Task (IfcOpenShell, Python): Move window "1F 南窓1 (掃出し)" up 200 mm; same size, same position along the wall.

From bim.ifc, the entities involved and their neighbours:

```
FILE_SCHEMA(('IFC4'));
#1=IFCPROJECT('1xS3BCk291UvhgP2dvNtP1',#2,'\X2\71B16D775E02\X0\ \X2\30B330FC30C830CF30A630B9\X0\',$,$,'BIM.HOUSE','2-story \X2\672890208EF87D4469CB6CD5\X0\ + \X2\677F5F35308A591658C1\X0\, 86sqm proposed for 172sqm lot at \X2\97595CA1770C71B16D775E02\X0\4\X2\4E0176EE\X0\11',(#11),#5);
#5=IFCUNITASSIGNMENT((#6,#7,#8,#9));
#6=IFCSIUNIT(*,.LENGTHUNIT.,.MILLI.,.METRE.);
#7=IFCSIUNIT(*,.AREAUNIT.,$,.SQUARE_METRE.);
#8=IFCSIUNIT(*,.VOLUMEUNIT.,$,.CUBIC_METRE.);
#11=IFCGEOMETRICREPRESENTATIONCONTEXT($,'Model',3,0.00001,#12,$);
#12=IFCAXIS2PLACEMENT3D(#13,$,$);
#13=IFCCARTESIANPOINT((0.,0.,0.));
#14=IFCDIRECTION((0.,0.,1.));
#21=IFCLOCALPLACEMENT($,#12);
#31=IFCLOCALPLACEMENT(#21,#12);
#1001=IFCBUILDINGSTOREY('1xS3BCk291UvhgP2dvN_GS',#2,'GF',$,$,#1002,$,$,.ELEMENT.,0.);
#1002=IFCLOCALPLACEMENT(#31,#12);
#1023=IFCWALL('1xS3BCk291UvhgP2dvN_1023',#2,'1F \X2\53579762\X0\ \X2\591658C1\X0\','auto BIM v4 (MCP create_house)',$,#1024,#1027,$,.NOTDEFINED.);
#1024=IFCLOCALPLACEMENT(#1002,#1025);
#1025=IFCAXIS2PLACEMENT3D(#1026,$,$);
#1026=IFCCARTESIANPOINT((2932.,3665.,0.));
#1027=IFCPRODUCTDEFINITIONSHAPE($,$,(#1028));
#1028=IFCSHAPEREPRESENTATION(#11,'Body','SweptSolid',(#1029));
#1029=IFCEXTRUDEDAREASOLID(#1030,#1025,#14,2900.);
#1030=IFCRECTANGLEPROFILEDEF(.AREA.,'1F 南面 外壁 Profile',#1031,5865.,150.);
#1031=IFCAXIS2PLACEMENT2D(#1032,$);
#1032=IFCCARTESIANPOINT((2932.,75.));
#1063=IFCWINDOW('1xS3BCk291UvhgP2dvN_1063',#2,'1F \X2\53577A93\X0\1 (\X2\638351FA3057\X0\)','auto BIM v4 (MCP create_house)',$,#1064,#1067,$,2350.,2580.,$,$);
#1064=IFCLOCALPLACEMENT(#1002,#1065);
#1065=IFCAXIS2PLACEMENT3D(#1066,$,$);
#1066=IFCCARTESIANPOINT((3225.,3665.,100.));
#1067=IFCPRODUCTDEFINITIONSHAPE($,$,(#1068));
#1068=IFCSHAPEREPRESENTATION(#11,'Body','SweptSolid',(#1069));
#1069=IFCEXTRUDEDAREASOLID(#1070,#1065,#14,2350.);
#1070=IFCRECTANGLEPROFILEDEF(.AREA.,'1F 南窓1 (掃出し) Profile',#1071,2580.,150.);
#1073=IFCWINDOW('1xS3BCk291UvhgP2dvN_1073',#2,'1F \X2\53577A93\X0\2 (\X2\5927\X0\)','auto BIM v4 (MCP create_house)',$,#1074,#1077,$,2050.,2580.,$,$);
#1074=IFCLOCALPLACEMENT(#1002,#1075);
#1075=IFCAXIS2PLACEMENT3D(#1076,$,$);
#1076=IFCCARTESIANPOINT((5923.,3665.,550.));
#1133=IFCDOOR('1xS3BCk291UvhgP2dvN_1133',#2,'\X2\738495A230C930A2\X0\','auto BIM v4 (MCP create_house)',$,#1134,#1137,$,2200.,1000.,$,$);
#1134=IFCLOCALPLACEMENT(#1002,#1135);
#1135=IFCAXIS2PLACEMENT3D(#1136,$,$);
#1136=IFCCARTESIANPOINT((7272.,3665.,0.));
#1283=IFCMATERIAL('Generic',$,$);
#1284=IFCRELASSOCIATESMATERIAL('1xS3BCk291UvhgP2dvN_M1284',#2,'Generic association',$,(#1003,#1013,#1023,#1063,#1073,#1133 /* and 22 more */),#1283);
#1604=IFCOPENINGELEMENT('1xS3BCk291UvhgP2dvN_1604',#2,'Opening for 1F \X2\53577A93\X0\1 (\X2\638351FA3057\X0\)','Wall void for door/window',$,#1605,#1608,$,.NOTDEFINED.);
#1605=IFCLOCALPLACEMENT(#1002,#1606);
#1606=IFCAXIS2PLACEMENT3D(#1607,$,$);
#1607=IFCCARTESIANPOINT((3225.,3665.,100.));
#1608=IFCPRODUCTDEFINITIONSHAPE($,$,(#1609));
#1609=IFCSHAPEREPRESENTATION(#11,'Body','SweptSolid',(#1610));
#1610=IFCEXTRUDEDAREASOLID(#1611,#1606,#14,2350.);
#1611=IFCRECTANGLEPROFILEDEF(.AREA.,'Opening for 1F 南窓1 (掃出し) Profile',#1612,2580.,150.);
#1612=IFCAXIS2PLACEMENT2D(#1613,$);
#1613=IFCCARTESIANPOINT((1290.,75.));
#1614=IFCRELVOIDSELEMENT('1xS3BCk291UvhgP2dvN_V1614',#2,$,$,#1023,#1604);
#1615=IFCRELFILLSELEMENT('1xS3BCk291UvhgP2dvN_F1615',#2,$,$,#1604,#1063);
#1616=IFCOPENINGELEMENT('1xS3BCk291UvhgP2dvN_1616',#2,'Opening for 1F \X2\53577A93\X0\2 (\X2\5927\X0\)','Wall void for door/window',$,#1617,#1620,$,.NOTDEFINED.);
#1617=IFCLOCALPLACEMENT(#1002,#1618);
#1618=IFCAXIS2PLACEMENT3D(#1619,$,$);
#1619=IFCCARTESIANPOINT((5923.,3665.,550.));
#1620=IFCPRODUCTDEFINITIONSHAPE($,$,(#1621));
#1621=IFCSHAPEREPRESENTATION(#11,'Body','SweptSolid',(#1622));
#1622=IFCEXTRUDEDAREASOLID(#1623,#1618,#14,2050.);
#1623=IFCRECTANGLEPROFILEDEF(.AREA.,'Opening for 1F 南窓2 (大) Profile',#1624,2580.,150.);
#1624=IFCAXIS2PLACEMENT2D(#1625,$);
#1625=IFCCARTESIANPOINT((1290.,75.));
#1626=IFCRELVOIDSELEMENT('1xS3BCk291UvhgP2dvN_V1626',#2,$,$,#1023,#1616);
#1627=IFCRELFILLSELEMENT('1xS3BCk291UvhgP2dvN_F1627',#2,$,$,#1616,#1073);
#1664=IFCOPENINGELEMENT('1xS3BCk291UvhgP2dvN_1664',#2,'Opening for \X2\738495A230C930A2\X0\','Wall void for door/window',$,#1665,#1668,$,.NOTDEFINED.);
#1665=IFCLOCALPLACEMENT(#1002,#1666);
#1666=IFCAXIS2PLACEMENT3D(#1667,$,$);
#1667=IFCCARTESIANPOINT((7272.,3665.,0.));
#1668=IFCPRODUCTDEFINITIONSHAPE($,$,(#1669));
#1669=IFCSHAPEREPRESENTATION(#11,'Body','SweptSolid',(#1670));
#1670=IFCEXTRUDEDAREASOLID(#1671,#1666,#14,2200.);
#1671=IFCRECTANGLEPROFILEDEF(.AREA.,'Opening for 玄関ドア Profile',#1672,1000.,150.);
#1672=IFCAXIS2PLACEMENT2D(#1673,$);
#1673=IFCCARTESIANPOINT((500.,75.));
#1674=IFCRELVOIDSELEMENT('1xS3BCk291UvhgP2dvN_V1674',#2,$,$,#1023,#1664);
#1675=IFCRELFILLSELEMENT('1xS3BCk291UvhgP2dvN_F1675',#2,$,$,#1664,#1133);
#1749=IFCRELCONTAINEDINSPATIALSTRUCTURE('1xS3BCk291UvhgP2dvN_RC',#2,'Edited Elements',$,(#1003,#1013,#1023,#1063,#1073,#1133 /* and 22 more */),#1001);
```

```python
import numpy as np
import ifcopenshell
import ifcopenshell.api.geometry
import ifcopenshell.util.placement
import ifcopenshell.util.unit

model = ifcopenshell.open("bim.ifc")
unit_scale = ifcopenshell.util.unit.calculate_unit_scale(model)

window = model.by_id(1063)
opening = window.FillsVoids[0].RelatingOpeningElement
dz = 200.0

shift = np.array([0.0, 0.0, dz])
# The window is not placed relative to its opening, so move both.
for product in (opening, window):
    matrix = ifcopenshell.util.placement.get_local_placement(product.ObjectPlacement)
    matrix[:3, 3] += shift
    ifcopenshell.api.geometry.edit_object_placement(model, product=product, matrix=matrix, is_si=False)

print(f"moved by {dz * unit_scale:+.3f} m")

model.write("bim_edited.ifc")
```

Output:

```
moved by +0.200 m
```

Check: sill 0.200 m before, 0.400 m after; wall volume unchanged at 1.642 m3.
